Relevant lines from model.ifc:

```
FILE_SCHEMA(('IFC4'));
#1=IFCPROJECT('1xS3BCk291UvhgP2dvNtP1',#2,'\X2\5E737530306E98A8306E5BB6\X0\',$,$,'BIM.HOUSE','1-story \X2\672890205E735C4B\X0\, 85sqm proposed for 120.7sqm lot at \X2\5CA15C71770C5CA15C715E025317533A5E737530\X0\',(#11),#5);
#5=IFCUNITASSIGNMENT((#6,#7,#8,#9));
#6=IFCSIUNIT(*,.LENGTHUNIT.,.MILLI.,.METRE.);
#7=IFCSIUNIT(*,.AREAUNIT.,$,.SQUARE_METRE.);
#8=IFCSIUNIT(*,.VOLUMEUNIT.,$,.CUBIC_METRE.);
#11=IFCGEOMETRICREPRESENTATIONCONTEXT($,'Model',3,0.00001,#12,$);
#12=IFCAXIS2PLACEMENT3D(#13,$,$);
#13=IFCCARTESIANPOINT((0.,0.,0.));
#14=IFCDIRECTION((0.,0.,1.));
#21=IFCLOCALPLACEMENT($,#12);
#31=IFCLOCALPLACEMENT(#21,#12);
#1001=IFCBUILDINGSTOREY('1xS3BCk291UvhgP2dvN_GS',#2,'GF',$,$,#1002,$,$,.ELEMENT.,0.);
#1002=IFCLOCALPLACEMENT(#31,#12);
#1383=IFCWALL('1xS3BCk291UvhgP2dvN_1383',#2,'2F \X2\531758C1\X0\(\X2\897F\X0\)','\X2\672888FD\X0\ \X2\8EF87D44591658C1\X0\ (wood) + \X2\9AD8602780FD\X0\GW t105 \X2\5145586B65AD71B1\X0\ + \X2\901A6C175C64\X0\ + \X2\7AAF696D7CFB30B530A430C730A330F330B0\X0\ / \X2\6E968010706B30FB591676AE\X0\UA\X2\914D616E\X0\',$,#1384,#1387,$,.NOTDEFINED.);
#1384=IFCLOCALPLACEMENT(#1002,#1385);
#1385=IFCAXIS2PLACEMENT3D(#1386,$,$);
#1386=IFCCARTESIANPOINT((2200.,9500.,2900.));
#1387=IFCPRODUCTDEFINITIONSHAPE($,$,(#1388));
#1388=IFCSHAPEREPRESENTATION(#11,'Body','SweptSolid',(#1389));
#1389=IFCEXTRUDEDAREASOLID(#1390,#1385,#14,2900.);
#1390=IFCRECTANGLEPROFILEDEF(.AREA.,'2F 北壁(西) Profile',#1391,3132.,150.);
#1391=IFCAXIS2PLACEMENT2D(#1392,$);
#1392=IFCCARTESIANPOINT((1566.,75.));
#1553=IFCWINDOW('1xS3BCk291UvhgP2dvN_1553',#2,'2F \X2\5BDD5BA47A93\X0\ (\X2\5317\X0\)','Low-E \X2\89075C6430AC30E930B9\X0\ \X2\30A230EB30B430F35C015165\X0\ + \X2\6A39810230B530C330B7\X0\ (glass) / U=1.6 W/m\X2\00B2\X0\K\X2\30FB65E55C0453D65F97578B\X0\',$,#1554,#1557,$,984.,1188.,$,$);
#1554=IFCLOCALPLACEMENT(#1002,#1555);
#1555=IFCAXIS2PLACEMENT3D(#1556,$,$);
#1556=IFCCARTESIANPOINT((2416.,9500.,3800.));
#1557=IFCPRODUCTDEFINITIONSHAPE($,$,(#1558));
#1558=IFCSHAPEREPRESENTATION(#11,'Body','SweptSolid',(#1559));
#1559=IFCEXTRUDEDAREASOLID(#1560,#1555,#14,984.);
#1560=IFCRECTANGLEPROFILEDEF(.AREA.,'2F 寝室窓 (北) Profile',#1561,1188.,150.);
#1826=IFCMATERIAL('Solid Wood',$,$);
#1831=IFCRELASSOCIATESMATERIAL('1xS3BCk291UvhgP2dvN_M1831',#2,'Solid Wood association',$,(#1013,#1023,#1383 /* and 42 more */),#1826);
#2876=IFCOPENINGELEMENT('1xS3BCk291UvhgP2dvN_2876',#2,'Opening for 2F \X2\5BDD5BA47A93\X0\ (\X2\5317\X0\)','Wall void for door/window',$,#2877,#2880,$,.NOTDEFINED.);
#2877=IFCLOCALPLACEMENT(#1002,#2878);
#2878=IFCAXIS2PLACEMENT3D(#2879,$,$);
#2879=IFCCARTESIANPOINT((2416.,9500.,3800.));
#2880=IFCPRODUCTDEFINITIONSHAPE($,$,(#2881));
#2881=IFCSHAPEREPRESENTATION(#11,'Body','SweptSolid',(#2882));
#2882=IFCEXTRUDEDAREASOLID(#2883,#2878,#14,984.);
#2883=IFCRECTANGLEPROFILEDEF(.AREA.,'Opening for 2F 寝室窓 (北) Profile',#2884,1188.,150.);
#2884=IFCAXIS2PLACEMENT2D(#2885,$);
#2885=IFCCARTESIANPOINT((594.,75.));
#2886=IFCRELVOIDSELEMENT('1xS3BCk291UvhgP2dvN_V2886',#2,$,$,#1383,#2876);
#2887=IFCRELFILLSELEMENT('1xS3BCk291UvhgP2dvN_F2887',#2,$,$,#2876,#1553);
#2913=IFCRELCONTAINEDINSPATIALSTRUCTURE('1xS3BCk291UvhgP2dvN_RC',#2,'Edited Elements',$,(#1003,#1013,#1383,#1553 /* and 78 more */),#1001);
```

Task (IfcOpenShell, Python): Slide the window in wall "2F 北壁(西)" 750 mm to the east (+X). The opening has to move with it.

```python
import ifcopenshell
import ifcopenshell.api.geometry
import ifcopenshell.util.placement
import ifcopenshell.util.unit

model = ifcopenshell.open("model.ifc")
unit_scale = ifcopenshell.util.unit.calculate_unit_scale(model)

window = model.by_guid("1xS3BCk291UvhgP2dvN_1553")
opening = window.FillsVoids[0].RelatingOpeningElement
wall = opening.VoidsElements[0].RelatingBuildingElement

wall_matrix = ifcopenshell.util.placement.get_local_placement(wall.ObjectPlacement)
shift = wall_matrix[:3, 0] * 0.75 / unit_scale
before = ifcopenshell.util.placement.get_local_placement(window.ObjectPlacement)[:3, 3].copy()

# The window is not placed relative to its opening, so move both.
for product in (opening, window):
    matrix = ifcopenshell.util.placement.get_local_placement(product.ObjectPlacement)
    matrix[:3, 3] += shift
    ifcopenshell.api.geometry.edit_object_placement(model, product=product, matrix=matrix, is_si=False)

after = ifcopenshell.util.placement.get_local_placement(window.ObjectPlacement)[:3, 3]
print("window moved by", (after - before).round(3) + 0.0)

model.write("model_rev.ifc")
```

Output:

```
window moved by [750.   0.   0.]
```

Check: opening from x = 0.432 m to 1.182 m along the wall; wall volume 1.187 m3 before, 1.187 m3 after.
